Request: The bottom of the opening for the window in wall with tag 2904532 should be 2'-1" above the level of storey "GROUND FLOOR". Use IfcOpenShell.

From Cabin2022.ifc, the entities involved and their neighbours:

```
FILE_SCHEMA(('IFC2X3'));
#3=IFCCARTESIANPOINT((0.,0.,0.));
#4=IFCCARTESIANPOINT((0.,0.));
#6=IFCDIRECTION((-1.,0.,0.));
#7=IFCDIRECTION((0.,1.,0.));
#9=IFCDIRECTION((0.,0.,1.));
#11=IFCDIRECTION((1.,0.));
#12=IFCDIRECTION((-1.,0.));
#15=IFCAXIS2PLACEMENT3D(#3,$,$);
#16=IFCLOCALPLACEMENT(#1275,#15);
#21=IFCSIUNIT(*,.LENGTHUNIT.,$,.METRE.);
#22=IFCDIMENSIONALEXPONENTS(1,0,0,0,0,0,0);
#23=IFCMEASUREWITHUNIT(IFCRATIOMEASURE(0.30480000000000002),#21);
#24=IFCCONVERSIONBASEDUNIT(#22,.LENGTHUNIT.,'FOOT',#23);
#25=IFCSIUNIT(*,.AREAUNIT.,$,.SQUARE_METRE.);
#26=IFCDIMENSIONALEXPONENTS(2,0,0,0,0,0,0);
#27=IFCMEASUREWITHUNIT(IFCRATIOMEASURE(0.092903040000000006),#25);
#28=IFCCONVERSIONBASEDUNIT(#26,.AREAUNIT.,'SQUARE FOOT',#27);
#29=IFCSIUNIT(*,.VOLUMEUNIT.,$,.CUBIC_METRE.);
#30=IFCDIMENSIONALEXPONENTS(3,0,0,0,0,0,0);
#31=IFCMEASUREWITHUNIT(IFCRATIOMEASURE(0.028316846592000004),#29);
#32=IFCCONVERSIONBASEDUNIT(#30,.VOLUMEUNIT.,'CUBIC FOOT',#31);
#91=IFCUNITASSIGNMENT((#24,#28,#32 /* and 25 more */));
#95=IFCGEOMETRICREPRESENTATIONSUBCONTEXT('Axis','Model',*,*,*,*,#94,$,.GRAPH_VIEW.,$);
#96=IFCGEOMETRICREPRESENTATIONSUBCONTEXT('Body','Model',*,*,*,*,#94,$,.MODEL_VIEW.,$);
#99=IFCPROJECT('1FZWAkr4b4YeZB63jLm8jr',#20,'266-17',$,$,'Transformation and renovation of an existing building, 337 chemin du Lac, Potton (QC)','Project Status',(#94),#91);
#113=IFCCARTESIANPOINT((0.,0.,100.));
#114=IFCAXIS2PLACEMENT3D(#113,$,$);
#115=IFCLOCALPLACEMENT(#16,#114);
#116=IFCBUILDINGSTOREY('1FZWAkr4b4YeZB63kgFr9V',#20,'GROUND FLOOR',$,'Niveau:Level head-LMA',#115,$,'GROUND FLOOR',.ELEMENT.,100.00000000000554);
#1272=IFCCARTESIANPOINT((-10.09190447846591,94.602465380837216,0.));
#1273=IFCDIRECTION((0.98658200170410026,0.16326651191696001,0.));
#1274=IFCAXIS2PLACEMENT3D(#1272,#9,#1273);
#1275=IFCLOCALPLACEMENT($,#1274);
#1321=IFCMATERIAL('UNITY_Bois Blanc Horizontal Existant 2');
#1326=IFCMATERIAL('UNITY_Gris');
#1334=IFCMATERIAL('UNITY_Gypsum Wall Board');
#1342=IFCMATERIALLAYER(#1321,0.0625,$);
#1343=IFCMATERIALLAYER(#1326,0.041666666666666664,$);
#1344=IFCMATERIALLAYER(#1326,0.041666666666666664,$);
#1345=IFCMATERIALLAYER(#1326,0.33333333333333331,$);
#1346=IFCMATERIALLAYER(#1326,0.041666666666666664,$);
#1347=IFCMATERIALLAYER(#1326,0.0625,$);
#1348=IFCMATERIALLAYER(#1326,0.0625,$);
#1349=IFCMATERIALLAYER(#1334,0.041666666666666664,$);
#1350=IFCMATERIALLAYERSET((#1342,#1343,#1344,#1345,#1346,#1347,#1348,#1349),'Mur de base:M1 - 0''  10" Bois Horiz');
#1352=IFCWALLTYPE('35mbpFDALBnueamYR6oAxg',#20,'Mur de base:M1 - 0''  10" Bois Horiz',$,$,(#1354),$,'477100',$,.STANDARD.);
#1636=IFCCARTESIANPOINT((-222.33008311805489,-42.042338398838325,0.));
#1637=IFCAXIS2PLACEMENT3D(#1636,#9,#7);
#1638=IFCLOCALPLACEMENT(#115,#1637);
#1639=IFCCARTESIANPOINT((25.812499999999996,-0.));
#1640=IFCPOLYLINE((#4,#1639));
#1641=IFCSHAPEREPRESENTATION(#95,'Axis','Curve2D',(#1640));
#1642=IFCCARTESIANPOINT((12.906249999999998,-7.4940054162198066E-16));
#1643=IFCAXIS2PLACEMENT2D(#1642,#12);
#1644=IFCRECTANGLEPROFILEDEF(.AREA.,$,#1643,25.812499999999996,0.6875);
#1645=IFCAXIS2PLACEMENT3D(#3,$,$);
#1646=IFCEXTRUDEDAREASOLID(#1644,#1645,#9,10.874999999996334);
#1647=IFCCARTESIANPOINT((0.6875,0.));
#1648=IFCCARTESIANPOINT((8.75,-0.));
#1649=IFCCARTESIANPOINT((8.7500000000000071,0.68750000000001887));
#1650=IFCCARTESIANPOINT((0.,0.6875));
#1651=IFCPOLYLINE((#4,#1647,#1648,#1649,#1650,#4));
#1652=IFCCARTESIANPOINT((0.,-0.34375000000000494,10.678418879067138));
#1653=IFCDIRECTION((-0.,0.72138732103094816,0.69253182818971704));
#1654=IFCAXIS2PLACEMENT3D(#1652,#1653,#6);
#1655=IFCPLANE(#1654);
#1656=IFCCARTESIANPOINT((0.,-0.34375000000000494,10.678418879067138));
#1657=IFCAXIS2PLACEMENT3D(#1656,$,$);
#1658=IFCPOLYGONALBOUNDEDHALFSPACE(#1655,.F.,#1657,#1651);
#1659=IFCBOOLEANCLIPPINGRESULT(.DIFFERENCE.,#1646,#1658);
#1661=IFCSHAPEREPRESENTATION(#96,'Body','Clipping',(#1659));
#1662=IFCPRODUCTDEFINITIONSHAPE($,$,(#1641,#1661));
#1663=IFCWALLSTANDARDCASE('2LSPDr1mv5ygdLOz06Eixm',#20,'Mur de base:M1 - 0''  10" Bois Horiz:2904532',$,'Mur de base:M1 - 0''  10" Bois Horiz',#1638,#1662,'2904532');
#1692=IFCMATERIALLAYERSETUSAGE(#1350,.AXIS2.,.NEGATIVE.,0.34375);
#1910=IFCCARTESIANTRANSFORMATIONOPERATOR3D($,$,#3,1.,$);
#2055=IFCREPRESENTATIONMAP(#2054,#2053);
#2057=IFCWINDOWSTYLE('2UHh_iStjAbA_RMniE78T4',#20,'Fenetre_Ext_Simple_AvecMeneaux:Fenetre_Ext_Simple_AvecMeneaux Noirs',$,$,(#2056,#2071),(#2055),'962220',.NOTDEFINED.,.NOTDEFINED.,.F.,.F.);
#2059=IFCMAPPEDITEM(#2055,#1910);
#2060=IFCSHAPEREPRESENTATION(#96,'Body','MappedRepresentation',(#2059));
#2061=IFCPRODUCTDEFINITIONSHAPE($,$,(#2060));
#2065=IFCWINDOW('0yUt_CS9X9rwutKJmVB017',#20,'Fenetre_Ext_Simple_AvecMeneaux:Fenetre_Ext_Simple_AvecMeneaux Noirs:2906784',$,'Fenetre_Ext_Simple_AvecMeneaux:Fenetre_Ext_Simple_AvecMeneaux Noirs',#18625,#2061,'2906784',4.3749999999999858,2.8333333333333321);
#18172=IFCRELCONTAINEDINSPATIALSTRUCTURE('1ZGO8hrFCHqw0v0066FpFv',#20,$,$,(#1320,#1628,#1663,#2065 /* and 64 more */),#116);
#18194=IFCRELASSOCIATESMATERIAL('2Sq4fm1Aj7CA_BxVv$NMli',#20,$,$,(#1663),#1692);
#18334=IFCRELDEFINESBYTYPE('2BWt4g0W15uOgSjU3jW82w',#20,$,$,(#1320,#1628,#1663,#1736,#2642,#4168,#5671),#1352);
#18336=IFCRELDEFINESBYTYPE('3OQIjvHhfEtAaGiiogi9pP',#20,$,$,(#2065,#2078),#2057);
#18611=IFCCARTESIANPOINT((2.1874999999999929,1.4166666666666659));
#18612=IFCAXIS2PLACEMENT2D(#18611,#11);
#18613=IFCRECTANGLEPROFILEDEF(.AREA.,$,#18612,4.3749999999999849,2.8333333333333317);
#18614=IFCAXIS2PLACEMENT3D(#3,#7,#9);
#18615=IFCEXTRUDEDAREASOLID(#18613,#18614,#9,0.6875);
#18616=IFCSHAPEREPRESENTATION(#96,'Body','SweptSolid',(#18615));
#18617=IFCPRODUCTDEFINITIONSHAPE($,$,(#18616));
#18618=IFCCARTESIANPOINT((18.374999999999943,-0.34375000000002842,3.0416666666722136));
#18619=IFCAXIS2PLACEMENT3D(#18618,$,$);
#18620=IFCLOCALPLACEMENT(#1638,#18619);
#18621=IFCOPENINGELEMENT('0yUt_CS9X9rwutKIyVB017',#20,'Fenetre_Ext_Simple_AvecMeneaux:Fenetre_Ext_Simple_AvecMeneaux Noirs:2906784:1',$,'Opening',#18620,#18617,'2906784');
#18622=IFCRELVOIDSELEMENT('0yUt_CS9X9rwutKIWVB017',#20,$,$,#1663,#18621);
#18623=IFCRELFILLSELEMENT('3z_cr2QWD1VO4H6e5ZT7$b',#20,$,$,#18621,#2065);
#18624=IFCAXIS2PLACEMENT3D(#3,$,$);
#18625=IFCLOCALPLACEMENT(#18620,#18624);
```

```python
import numpy as np
import ifcopenshell
import ifcopenshell.api.geometry
import ifcopenshell.geom
import ifcopenshell.util.element
import ifcopenshell.util.placement
import ifcopenshell.util.shape
import ifcopenshell.util.unit

model = ifcopenshell.open("Cabin2022.ifc")
unit_scale = ifcopenshell.util.unit.calculate_unit_scale(model)

window = model.by_guid("0yUt_CS9X9rwutKJmVB017")
opening = window.FillsVoids[0].RelatingOpeningElement
storey = ifcopenshell.util.element.get_container(window, ifc_class="IfcBuildingStorey")
level = ifcopenshell.util.placement.get_local_placement(storey.ObjectPlacement)[2, 3]

# The opening's origin need not be at the sill, so measure its lowest point.
shape = ifcopenshell.geom.create_shape(ifcopenshell.geom.settings(), opening)
bottom = ifcopenshell.util.shape.get_shape_bottom_elevation(shape, shape.geometry) / unit_scale
dz = level + 25 * 0.0254 / unit_scale - bottom

shift = np.array([0.0, 0.0, dz])
# The window is placed relative to its opening, so it follows when the opening moves.
matrix = ifcopenshell.util.placement.get_local_placement(opening.ObjectPlacement)
matrix[:3, 3] += shift
ifcopenshell.api.geometry.edit_object_placement(
    model, product=opening, matrix=matrix, is_si=False, should_transform_children=True
)

print(f"moved by {dz * unit_scale:+.3f} m")

model.write("Cabin2022_rev.ifc")
```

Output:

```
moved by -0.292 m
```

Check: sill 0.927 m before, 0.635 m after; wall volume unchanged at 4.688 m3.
